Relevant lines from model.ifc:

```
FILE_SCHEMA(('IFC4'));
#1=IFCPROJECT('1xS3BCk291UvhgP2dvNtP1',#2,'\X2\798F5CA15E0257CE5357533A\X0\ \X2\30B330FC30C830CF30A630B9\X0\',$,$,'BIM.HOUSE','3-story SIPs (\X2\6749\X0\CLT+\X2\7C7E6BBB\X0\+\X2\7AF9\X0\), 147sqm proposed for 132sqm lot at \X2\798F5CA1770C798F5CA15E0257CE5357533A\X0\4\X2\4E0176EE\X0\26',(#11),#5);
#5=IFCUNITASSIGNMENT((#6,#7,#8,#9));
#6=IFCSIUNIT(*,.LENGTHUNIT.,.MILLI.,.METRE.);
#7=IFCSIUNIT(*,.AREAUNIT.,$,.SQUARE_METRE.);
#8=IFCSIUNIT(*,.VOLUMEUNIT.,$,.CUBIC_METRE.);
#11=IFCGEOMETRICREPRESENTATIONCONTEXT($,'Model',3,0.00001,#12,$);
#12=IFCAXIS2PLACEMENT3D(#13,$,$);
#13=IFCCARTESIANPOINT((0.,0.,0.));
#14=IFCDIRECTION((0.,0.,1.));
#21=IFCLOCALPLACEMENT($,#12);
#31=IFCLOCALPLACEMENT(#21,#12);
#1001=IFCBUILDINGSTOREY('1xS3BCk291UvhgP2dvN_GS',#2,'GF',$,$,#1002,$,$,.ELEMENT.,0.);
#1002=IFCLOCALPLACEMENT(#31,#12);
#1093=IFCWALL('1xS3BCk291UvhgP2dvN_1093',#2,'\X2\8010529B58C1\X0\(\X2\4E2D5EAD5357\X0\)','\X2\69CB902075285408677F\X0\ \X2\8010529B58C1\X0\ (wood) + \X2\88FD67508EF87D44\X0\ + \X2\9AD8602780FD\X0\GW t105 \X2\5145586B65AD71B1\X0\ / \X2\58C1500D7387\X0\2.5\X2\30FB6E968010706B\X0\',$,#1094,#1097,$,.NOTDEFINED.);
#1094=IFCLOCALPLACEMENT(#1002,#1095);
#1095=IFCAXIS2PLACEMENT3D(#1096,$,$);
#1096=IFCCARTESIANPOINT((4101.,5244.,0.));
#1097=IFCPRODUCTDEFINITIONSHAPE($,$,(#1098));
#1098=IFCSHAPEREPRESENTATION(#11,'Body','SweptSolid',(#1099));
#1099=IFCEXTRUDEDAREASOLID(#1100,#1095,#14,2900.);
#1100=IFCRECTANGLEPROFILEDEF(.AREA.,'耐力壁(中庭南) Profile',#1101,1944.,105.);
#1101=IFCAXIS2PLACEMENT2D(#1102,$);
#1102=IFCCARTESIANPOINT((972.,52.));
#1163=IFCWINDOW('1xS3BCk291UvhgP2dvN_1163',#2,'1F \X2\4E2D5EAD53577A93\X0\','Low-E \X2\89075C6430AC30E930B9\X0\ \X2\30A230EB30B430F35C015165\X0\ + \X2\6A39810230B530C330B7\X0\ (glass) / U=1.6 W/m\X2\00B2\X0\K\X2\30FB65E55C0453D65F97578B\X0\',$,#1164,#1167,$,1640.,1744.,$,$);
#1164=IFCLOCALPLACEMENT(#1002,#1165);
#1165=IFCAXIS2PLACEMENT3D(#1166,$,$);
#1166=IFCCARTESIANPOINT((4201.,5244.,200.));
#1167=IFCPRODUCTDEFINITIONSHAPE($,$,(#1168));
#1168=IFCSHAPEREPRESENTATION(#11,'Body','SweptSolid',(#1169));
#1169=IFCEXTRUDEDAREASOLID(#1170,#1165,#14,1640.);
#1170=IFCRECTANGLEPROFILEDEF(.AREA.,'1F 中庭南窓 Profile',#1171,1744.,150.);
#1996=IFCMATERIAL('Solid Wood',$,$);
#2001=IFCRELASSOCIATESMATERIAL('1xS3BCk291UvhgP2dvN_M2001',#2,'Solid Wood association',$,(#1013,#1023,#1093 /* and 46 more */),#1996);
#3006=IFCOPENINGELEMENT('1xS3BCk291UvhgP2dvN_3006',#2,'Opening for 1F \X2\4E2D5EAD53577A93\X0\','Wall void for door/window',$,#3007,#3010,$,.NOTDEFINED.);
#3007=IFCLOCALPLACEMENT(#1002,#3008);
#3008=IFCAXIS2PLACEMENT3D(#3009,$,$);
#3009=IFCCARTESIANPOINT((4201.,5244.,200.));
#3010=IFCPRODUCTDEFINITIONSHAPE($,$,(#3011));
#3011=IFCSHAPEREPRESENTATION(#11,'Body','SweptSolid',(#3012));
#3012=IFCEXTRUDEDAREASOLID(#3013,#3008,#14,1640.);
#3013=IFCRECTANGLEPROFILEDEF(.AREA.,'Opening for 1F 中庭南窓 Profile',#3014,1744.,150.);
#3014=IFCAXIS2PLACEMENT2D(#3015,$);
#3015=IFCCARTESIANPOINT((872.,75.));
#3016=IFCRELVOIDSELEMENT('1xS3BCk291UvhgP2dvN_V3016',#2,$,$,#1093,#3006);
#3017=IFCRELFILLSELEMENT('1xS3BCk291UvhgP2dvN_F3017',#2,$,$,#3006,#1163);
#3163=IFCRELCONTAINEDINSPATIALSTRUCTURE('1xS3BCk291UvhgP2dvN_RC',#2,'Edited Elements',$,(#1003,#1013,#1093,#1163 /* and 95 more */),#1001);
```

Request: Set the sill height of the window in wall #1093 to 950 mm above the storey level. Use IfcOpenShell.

```python
import numpy as np
import ifcopenshell
import ifcopenshell.api.geometry
import ifcopenshell.geom
import ifcopenshell.util.element
import ifcopenshell.util.placement
import ifcopenshell.util.shape
import ifcopenshell.util.unit

model = ifcopenshell.open("model.ifc")
unit_scale = ifcopenshell.util.unit.calculate_unit_scale(model)

window = model.by_guid("1xS3BCk291UvhgP2dvN_1163")
opening = window.FillsVoids[0].RelatingOpeningElement
storey = ifcopenshell.util.element.get_container(window, ifc_class="IfcBuildingStorey")
level = ifcopenshell.util.placement.get_local_placement(storey.ObjectPlacement)[2, 3]

# The opening's origin need not be at the sill, so measure its lowest point.
shape = ifcopenshell.geom.create_shape(ifcopenshell.geom.settings(), opening)
bottom = ifcopenshell.util.shape.get_shape_bottom_elevation(shape, shape.geometry) / unit_scale
dz = level + 0.95 / unit_scale - bottom

shift = np.array([0.0, 0.0, dz])
# The window is not placed relative to its opening, so move both.
for product in (opening, window):
    matrix = ifcopenshell.util.placement.get_local_placement(product.ObjectPlacement)
    matrix[:3, 3] += shift
    ifcopenshell.api.geometry.edit_object_placement(model, product=product, matrix=matrix, is_si=False)

print(f"moved by {dz * unit_scale:+.3f} m")

model.write("model_v2.ifc")
```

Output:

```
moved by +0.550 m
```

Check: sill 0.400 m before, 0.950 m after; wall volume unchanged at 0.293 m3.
